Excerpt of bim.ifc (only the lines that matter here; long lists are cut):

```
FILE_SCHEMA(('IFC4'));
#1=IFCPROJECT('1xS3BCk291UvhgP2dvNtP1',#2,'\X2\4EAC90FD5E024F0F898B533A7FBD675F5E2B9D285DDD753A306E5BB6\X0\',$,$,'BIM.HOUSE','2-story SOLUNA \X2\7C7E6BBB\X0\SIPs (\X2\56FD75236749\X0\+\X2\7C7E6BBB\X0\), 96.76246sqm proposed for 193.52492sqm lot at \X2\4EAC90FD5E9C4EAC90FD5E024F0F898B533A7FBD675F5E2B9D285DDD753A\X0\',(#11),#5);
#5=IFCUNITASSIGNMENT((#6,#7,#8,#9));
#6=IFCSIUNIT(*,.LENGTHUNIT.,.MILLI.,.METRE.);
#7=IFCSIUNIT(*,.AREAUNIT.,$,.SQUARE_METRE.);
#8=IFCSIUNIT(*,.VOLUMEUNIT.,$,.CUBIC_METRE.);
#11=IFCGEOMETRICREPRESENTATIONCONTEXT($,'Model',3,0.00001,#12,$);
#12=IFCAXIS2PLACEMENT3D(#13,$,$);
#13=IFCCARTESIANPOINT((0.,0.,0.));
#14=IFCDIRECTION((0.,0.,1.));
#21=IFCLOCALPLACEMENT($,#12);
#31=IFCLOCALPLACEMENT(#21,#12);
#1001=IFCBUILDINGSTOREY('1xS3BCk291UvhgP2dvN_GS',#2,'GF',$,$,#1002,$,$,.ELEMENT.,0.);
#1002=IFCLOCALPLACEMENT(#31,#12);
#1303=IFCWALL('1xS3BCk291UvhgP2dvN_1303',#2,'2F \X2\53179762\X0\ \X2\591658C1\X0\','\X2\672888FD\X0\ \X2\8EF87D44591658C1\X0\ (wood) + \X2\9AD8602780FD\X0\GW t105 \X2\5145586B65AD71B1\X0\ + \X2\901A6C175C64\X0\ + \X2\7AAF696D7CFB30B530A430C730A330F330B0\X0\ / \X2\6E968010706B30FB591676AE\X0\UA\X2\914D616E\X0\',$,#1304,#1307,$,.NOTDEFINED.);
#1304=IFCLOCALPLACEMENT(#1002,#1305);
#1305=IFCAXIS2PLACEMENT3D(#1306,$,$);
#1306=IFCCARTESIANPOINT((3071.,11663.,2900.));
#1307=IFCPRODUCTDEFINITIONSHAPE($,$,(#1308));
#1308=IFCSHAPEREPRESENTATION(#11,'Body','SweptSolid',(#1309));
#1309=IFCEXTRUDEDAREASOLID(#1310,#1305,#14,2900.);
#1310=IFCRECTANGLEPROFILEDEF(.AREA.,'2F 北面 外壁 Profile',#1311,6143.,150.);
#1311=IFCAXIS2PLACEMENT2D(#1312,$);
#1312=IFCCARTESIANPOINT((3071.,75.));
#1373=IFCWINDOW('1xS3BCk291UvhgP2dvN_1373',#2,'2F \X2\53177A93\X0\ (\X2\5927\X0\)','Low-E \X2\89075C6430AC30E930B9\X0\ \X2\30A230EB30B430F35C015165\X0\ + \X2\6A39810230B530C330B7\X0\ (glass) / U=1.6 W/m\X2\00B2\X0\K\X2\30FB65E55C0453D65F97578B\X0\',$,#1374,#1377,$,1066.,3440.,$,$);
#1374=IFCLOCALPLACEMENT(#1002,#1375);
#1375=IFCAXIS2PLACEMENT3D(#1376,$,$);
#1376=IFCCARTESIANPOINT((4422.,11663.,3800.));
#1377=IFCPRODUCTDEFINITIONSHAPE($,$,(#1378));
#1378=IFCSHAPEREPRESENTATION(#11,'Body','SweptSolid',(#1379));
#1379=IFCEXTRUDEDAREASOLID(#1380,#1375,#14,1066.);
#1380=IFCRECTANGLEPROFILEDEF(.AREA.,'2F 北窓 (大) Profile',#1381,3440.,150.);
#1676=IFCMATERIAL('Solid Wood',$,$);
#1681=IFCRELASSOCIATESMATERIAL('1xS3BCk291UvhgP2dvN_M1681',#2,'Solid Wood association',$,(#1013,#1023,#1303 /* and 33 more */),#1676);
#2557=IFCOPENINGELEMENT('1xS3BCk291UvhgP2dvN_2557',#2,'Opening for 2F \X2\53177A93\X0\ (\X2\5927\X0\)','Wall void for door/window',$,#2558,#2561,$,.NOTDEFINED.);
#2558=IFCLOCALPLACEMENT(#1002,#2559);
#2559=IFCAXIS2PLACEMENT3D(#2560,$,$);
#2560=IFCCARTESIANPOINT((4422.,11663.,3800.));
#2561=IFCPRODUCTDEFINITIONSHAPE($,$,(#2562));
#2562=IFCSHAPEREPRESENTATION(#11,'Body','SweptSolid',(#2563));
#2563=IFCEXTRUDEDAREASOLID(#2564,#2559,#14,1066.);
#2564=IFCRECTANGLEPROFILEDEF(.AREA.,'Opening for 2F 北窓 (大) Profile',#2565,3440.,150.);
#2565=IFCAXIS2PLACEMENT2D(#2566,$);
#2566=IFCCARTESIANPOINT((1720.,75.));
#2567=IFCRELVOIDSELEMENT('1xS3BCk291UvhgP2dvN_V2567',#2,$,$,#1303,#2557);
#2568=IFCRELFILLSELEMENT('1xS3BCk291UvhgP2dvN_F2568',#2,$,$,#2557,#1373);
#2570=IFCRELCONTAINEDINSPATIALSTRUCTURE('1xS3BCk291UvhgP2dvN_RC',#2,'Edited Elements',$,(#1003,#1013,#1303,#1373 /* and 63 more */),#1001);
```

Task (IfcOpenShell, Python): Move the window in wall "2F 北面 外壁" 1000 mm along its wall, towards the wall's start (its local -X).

```python
import ifcopenshell
import ifcopenshell.api.geometry
import ifcopenshell.util.placement

model = ifcopenshell.open("bim.ifc")

window = model.by_guid("1xS3BCk291UvhgP2dvN_1373")
opening = window.FillsVoids[0].RelatingOpeningElement
wall = opening.VoidsElements[0].RelatingBuildingElement

wall_matrix = ifcopenshell.util.placement.get_local_placement(wall.ObjectPlacement)
shift = wall_matrix[:3, 0] * -1000.0
before = ifcopenshell.util.placement.get_local_placement(window.ObjectPlacement)[:3, 3].copy()

# The window is not placed relative to its opening, so move both.
for product in (opening, window):
    matrix = ifcopenshell.util.placement.get_local_placement(product.ObjectPlacement)
    matrix[:3, 3] += shift
    ifcopenshell.api.geometry.edit_object_placement(model, product=product, matrix=matrix, is_si=False)

after = ifcopenshell.util.placement.get_local_placement(window.ObjectPlacement)[:3, 3]
print("window moved by", (after - before).round(3) + 0.0)

model.write("bim_v2.ifc")
```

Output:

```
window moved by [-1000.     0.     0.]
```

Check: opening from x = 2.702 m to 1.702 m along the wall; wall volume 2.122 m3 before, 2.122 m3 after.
